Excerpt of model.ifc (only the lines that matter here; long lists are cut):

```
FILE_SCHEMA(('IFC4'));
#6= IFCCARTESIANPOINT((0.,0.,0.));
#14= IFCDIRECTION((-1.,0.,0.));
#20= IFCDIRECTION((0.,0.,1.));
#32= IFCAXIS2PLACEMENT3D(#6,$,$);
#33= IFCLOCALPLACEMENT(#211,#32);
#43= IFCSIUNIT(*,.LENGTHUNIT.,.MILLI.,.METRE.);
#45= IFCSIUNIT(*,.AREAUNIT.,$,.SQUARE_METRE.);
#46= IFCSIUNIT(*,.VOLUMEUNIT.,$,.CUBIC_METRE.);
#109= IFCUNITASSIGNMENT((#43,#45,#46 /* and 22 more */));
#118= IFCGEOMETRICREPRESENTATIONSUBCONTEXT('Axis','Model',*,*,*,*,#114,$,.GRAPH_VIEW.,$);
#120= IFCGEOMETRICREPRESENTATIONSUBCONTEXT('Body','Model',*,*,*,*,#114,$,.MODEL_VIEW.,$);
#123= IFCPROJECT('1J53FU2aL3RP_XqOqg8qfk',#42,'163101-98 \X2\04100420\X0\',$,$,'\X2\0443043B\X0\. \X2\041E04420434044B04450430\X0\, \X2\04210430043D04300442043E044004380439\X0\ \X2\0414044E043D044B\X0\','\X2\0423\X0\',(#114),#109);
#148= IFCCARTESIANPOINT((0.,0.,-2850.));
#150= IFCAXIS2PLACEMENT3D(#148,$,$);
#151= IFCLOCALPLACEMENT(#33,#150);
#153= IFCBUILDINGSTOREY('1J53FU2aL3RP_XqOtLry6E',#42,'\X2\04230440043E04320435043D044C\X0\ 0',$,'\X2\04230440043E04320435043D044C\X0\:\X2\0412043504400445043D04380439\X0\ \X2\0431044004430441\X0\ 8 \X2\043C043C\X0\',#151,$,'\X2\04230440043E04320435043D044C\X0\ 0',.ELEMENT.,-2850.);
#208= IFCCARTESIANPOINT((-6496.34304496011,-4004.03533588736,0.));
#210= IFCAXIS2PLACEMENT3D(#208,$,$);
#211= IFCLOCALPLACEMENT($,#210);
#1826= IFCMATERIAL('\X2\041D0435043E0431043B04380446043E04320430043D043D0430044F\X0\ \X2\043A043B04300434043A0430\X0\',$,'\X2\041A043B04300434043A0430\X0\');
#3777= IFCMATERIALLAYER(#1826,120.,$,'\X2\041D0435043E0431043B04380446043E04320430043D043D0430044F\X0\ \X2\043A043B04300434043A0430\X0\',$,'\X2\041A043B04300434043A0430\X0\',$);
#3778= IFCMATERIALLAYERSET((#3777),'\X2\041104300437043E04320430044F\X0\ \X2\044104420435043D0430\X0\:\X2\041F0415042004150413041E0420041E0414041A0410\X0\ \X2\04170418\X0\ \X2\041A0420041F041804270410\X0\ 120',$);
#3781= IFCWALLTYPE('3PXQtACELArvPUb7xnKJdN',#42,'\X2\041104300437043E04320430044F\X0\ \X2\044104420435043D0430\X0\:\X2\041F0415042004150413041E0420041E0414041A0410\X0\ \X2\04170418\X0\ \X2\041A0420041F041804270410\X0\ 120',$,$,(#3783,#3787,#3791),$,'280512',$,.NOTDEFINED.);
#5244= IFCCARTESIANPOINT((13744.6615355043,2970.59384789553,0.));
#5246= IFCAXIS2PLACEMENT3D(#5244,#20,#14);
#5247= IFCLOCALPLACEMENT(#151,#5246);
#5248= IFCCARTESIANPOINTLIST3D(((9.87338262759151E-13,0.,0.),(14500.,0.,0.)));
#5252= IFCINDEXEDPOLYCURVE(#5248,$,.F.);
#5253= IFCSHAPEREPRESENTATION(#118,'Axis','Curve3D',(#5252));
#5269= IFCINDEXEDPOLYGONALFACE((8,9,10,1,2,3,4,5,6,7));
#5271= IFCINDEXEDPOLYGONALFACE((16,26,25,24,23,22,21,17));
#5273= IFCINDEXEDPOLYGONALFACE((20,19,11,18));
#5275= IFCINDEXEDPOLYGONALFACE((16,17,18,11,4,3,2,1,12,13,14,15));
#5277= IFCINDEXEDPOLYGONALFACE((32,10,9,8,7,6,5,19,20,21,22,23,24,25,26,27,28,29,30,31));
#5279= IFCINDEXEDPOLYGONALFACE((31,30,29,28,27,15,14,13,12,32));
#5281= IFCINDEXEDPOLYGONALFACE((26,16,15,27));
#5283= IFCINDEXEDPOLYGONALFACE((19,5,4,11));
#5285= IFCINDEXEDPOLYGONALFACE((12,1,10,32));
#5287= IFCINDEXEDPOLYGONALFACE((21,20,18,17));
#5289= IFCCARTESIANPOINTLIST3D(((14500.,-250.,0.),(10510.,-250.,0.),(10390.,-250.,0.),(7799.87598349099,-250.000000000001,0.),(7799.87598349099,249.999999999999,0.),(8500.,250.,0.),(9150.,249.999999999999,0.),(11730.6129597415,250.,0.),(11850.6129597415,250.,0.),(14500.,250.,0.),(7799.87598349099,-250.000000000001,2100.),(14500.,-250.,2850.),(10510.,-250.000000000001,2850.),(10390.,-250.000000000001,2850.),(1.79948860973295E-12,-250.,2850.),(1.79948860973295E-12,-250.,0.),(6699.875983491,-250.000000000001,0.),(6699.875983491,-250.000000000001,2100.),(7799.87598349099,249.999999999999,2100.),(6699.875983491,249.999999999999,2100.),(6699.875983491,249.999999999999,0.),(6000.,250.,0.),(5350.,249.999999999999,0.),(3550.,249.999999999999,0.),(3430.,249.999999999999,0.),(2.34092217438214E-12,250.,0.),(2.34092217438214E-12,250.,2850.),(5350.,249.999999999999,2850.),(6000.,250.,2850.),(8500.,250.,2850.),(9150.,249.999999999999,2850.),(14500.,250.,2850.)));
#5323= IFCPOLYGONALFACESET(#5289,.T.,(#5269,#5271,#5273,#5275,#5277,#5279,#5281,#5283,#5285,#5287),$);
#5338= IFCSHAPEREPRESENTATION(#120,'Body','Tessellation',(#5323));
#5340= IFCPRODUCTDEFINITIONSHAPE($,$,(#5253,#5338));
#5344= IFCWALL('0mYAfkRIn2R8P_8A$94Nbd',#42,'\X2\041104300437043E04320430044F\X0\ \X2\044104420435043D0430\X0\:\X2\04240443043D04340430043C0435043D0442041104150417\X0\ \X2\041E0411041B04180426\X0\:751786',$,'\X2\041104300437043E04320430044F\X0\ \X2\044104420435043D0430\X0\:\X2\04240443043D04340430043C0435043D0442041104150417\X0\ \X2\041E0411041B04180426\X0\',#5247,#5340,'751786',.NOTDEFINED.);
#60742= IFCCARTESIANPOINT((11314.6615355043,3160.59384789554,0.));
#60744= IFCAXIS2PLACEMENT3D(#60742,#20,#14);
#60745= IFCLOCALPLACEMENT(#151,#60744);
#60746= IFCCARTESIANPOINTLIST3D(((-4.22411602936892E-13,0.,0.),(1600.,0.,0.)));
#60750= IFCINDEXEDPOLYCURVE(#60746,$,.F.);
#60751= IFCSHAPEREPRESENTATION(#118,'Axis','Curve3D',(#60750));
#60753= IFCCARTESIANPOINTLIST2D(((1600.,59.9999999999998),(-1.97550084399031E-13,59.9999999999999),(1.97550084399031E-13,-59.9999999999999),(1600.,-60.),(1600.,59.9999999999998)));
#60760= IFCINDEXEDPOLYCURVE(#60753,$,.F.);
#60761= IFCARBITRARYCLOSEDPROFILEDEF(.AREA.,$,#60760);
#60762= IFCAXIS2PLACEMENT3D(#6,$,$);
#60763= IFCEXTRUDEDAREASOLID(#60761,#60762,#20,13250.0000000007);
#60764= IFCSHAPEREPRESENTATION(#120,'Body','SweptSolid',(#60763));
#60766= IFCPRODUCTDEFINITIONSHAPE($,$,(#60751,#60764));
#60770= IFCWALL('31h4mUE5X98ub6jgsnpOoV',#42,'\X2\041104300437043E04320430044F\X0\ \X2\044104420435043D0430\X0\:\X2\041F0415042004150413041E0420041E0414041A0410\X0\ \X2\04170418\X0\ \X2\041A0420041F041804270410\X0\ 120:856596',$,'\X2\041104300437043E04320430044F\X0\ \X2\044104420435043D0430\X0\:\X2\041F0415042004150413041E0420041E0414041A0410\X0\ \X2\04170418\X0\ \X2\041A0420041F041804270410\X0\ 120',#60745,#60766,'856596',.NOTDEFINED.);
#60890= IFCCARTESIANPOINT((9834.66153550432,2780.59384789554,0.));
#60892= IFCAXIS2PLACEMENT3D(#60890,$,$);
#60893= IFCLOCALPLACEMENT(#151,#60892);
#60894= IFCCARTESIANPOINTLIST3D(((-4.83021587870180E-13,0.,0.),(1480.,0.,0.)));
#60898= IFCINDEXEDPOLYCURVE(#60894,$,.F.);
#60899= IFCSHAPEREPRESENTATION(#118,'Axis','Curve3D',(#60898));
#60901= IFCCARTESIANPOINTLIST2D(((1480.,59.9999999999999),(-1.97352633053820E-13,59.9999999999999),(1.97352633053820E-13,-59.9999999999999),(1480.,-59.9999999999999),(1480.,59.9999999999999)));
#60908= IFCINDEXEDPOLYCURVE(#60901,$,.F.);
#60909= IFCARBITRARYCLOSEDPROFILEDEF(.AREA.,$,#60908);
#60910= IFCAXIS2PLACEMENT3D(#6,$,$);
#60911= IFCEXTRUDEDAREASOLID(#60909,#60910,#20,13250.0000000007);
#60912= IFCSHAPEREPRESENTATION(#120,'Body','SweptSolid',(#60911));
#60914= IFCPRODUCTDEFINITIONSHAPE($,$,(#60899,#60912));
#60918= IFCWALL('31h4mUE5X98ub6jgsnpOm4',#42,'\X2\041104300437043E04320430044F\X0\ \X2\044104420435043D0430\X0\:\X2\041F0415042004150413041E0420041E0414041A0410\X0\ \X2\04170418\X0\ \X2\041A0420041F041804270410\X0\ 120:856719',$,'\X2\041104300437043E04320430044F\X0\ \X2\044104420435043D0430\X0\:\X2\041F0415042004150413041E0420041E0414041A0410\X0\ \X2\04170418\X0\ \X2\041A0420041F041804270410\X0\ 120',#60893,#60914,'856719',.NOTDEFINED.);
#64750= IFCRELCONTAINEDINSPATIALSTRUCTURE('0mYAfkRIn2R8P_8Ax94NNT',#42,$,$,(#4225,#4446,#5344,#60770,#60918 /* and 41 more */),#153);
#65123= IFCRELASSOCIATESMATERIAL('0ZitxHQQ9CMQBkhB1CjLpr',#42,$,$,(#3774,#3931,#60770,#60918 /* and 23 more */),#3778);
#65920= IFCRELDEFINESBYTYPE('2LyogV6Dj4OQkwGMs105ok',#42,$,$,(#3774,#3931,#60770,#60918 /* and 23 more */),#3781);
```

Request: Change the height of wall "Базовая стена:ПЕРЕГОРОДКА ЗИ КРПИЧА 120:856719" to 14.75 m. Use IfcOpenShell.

```python
import ifcopenshell
import ifcopenshell.geom
import ifcopenshell.util.representation
import ifcopenshell.util.shape
import ifcopenshell.util.unit

model = ifcopenshell.open("model.ifc")
unit_scale = ifcopenshell.util.unit.calculate_unit_scale(model)
settings = ifcopenshell.geom.settings()


def volume(element):
    """Net volume in cubic metres, openings subtracted."""
    shape = ifcopenshell.geom.create_shape(settings, element)
    return ifcopenshell.util.shape.get_volume(shape.geometry)


wall = model.by_guid("31h4mUE5X98ub6jgsnpOm4")
before = volume(wall)

body = ifcopenshell.util.representation.get_representation(wall, "Model", "Body")
solid = body.Items[0]
old_height = solid.Depth
solid.Depth = 14.75 / unit_scale
after = volume(wall)

print(f"height {old_height:g} -> {solid.Depth:g}, volume {before:.3f} -> {after:.3f} m3")

model.write("model_updated.ifc")
```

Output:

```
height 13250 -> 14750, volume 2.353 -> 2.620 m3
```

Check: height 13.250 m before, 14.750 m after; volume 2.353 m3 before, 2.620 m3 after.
